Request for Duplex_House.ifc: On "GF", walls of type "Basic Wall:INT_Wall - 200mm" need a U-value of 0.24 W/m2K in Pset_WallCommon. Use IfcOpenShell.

First a look at what the model holds.

```python
import ifcopenshell
import ifcopenshell.util.element

model = ifcopenshell.open("Duplex_House.ifc")
print(model.schema)
storey = next(s for s in model.by_type("IfcBuildingStorey") if s.Name == "GF")
walls = [e for e in ifcopenshell.util.element.get_decomposition(storey) if e.is_a("IfcWall")]
seen = {}
for e in walls:
    element_type = ifcopenshell.util.element.get_type(e)
    key = (element_type.Name if element_type != e and element_type else None, ifcopenshell.util.element.get_pset(e, "Pset_WallCommon", "ThermalTransmittance"))
    seen[key] = seen.get(key, 0) + 1
for (name, value), count in sorted(seen.items(), key=str):
    print(count, "x", name, "|", value)
```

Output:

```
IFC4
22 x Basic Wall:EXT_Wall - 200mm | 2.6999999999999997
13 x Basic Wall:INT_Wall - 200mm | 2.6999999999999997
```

```python
import ifcopenshell
import ifcopenshell.api.pset
import ifcopenshell.util.element

model = ifcopenshell.open("Duplex_House.ifc")

storey = next(s for s in model.by_type("IfcBuildingStorey") if s.Name == "GF")
walls = [e for e in ifcopenshell.util.element.get_decomposition(storey) if e.is_a("IfcWall")]

count = 0
for e in walls:
    element_type = ifcopenshell.util.element.get_type(e)
    if element_type in (None, e) or element_type.Name != "Basic Wall:INT_Wall - 200mm":
        continue
    # add_pset returns the element's existing set when there is one.
    pset = ifcopenshell.api.pset.add_pset(model, product=e, name="Pset_WallCommon")
    ifcopenshell.api.pset.edit_pset(model, pset=pset, properties={"ThermalTransmittance": 0.24})
    count += 1

print(count, "walls updated")

model.write("Duplex_House-out.ifc")
```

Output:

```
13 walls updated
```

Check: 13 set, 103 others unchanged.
